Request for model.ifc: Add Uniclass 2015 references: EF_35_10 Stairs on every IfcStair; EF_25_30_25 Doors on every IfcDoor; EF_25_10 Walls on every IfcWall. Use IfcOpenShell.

First a look at what the model holds.

```python
import ifcopenshell

model = ifcopenshell.open("model.ifc")
print(model.schema)
print("classifications:", [c.Name for c in model.by_type("IfcClassification")])
for ifc_class in ("IfcDoor", "IfcRoof", "IfcStair", "IfcWall", "IfcWindow"):
    print(ifc_class, len(model.by_type(ifc_class)))
```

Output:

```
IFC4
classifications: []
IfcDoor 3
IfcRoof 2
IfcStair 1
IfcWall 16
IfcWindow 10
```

```python
import ifcopenshell
import ifcopenshell.api.classification

model = ifcopenshell.open("model.ifc")

system = ifcopenshell.api.classification.add_classification(model, classification="Uniclass 2015")

codes = {
    "IfcStair": ("EF_35_10", "Stairs"),
    "IfcDoor": ("EF_25_30_25", "Doors"),
    "IfcWall": ("EF_25_10", "Walls"),
}
for ifc_class, (code, name) in codes.items():
    products = model.by_type(ifc_class)
    ifcopenshell.api.classification.add_reference(
        model, products=products, classification=system, identification=code, name=name
    )
    print(code, len(products))

model.write("model_v2.ifc")
```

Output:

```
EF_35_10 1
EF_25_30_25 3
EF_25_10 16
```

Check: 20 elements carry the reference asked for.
